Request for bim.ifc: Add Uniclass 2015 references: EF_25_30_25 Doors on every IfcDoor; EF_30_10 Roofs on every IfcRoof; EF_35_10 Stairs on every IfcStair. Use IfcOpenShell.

First a look at what the model holds.

```python
import ifcopenshell

model = ifcopenshell.open("bim.ifc")
print(model.schema)
print("classifications:", [c.Name for c in model.by_type("IfcClassification")])
for ifc_class in ("IfcDoor", "IfcRoof", "IfcStair", "IfcWall", "IfcWindow"):
    print(ifc_class, len(model.by_type(ifc_class)))
```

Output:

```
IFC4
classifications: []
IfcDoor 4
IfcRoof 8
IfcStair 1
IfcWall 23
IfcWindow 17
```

```python
import ifcopenshell
import ifcopenshell.api.classification

model = ifcopenshell.open("bim.ifc")

system = ifcopenshell.api.classification.add_classification(model, classification="Uniclass 2015")

codes = {
    "IfcDoor": ("EF_25_30_25", "Doors"),
    "IfcRoof": ("EF_30_10", "Roofs"),
    "IfcStair": ("EF_35_10", "Stairs"),
}
for ifc_class, (code, name) in codes.items():
    products = model.by_type(ifc_class)
    ifcopenshell.api.classification.add_reference(
        model, products=products, classification=system, identification=code, name=name
    )
    print(code, len(products))

model.write("bim_rev.ifc")
```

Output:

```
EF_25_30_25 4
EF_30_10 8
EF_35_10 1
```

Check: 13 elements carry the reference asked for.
